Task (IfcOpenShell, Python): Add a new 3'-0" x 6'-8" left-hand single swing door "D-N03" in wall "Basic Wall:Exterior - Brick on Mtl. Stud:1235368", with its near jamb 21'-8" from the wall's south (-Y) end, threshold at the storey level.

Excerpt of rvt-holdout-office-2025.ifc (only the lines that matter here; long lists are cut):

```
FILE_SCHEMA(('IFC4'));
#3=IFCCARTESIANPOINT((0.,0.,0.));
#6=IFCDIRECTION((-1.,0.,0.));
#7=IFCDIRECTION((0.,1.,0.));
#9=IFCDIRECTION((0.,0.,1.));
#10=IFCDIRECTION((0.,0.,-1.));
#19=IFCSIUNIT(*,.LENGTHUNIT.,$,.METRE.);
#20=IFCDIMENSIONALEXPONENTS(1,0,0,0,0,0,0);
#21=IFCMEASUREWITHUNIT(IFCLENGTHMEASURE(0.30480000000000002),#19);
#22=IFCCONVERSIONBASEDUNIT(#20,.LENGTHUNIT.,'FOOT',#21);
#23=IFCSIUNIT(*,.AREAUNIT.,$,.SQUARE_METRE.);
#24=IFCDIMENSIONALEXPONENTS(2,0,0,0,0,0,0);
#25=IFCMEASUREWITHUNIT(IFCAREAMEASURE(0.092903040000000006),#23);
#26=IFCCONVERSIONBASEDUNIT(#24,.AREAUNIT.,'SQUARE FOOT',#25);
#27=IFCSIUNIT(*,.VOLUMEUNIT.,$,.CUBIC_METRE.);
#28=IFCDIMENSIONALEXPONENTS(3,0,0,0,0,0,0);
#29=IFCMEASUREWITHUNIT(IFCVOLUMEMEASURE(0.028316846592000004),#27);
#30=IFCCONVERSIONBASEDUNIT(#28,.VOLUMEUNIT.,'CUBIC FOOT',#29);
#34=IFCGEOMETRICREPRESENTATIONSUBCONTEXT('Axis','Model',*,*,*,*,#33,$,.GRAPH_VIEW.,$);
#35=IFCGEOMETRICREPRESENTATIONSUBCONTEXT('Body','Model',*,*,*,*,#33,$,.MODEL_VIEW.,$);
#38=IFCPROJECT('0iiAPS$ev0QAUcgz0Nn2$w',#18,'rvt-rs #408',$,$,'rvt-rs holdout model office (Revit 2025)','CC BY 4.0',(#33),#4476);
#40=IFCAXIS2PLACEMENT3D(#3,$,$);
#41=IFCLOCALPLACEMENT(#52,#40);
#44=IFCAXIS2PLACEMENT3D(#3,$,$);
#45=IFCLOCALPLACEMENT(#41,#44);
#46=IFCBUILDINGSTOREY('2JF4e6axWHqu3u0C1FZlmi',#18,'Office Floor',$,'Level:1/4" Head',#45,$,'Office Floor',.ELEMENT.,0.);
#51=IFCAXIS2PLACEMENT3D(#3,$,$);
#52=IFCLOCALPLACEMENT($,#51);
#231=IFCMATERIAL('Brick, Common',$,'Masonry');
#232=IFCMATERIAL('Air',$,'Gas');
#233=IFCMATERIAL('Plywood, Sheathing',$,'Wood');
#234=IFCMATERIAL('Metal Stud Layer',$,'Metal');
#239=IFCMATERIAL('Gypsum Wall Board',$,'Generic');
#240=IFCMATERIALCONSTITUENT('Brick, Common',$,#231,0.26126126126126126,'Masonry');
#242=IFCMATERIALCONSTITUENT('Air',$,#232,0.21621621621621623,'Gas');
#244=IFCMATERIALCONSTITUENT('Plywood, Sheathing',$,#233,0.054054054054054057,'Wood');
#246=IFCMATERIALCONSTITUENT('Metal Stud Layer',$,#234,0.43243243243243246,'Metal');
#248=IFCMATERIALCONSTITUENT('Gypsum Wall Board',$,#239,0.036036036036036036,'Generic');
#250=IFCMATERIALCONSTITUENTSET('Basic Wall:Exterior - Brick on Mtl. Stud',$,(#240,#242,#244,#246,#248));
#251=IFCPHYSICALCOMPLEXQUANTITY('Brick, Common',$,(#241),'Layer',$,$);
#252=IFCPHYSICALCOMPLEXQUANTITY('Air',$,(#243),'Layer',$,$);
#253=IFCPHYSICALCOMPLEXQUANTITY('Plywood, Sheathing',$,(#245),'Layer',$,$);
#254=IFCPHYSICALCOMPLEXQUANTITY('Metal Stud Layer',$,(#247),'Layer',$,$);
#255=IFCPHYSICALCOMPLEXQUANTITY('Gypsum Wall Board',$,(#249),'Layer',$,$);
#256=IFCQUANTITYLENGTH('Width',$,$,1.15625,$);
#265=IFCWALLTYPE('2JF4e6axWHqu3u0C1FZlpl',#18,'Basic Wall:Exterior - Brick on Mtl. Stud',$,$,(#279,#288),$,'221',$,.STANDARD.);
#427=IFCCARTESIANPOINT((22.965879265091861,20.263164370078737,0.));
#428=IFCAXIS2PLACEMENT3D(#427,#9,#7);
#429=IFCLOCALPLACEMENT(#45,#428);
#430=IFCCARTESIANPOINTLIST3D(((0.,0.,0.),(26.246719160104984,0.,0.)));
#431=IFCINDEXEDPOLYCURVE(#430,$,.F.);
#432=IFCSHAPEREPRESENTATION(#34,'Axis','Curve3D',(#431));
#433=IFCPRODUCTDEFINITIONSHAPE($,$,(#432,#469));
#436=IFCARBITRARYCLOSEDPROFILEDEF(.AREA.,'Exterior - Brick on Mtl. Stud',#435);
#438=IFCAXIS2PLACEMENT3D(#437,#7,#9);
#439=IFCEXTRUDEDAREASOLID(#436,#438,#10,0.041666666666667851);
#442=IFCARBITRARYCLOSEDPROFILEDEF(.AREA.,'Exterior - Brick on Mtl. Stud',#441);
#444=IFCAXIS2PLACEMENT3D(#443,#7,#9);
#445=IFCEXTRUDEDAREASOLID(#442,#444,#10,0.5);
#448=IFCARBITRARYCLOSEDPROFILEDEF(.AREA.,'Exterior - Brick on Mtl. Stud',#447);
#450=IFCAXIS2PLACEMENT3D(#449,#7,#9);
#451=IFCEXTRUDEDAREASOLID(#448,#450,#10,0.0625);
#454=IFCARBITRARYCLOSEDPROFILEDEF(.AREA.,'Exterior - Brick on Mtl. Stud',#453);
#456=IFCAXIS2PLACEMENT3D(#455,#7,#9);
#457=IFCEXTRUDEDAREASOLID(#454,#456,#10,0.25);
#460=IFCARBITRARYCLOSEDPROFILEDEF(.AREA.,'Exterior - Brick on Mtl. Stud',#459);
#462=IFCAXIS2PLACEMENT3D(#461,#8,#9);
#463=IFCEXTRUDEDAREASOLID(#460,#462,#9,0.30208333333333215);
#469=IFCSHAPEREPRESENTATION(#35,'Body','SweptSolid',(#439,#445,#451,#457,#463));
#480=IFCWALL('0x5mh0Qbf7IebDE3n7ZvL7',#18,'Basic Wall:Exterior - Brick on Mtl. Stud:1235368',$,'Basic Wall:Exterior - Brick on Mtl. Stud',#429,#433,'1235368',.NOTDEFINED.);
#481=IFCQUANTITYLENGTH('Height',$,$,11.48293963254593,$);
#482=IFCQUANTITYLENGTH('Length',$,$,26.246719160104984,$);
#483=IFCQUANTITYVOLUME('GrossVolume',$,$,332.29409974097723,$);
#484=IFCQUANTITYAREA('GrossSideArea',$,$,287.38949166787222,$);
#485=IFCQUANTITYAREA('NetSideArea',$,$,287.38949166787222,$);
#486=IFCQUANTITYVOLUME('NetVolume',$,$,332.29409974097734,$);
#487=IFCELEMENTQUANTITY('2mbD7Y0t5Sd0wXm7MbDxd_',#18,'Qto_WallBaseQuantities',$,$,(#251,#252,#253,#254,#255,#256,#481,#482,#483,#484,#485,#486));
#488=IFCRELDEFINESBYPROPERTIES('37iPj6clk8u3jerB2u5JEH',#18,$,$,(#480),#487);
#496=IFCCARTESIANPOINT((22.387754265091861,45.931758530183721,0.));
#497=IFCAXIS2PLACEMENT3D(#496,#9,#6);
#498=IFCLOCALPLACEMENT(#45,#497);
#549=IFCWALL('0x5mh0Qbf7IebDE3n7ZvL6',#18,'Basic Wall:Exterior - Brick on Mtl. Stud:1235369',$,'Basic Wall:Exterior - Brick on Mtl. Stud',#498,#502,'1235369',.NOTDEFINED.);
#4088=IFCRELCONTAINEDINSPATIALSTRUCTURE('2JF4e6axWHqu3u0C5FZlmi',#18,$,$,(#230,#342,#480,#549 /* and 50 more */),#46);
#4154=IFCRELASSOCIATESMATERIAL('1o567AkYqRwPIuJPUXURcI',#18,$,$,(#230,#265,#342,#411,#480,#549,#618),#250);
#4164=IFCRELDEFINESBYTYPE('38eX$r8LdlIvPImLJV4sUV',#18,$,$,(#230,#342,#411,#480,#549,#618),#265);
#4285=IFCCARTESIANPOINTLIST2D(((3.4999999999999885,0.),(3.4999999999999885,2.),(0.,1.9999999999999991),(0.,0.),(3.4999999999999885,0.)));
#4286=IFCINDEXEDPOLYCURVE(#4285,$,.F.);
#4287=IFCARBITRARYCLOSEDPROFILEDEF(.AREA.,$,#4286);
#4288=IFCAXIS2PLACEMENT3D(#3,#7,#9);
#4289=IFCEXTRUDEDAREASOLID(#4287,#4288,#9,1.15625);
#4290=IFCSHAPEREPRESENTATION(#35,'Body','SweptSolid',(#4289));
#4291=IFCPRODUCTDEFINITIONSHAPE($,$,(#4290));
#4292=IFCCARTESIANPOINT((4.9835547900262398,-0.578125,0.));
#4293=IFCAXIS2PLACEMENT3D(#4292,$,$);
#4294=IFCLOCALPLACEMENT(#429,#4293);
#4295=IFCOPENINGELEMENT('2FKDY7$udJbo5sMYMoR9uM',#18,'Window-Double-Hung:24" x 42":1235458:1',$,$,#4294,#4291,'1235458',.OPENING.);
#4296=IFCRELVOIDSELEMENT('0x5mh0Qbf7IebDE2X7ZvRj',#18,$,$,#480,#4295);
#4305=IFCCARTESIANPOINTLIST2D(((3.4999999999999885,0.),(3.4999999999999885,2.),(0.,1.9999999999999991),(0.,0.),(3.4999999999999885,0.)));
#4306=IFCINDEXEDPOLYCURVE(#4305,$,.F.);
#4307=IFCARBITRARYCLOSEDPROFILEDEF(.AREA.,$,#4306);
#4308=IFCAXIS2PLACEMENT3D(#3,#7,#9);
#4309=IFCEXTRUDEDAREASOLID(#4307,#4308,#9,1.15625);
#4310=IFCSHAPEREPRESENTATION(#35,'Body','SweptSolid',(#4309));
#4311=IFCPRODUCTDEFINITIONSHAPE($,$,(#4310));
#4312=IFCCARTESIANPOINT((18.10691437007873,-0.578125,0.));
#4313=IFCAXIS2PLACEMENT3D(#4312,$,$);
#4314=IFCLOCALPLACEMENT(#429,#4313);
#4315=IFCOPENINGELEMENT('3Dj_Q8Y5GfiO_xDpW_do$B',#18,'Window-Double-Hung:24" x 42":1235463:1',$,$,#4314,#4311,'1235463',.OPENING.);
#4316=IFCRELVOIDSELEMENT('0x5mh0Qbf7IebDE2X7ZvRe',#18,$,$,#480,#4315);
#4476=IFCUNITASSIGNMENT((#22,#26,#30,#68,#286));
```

```python
import numpy as np
import ifcopenshell
import ifcopenshell.api.feature
import ifcopenshell.api.geometry
import ifcopenshell.api.pset
import ifcopenshell.api.root
import ifcopenshell.api.spatial
import ifcopenshell.geom
import ifcopenshell.util.element
import ifcopenshell.util.placement
import ifcopenshell.util.representation
import ifcopenshell.util.shape
import ifcopenshell.util.unit

model = ifcopenshell.open("rvt-holdout-office-2025.ifc")
unit_scale = ifcopenshell.util.unit.calculate_unit_scale(model)
area_scale = ifcopenshell.util.unit.calculate_unit_scale(model, "AREAUNIT")
volume_scale = ifcopenshell.util.unit.calculate_unit_scale(model, "VOLUMEUNIT")
settings = ifcopenshell.geom.settings()


def volume(element):
    """Net volume in cubic metres, openings subtracted."""
    shape = ifcopenshell.geom.create_shape(settings, element)
    return ifcopenshell.util.shape.get_volume(shape.geometry)


wall = model.by_id(480)
storey = ifcopenshell.util.element.get_container(wall, ifc_class="IfcBuildingStorey")
context = ifcopenshell.util.representation.get_context(model, "Model", "Body", "MODEL_VIEW")
before = volume(wall)

width, height, from_end, sill = 0.9144, 2.032, 6.604, 0.0  # metres

# The wall runs along its own X axis, and the end named is its -X end.
wall_shape = ifcopenshell.geom.create_shape(settings, wall)
x, y, z = ifcopenshell.util.shape.get_vertices(wall_shape.geometry).T
start = x.min() + from_end
face, thickness = float(y.min()), float(y.max() - y.min())
wall_matrix = ifcopenshell.util.placement.get_local_placement(wall.ObjectPlacement)
level = ifcopenshell.util.placement.get_local_placement(storey.ObjectPlacement)[2, 3]


def in_wall(x, y):
    """Placement at x, y metres in the wall's axes, at sill height."""
    matrix = wall_matrix.copy()
    matrix[:, 3] = wall_matrix @ np.array([x / unit_scale, y / unit_scale, 0.0, 1.0])
    matrix[2, 3] = level + sill / unit_scale
    return matrix


# Opening: a box that overshoots both wall faces by 50 mm.
opening = ifcopenshell.api.root.create_entity(model, ifc_class="IfcOpeningElement", predefined_type="OPENING")
box = ifcopenshell.api.geometry.add_wall_representation(
    model, context=context, length=width, height=height, thickness=thickness + 0.1
)
ifcopenshell.api.geometry.assign_representation(model, product=opening, representation=box)
ifcopenshell.api.geometry.edit_object_placement(model, product=opening, matrix=in_wall(start, face - 0.05), is_si=False)
ifcopenshell.api.feature.add_feature(model, feature=opening, element=wall)

door = ifcopenshell.api.root.create_entity(model, ifc_class="IfcDoor", name="D-N03", predefined_type="DOOR")
door.OverallWidth, door.OverallHeight = width / unit_scale, height / unit_scale
door.OperationType = "SINGLE_SWING_LEFT"
body = ifcopenshell.api.geometry.add_door_representation(
    model,
    context=context,
    overall_width=door.OverallWidth,
    overall_height=door.OverallHeight,
    operation_type="SINGLE_SWING_LEFT",
    lining_properties={"LiningDepth": thickness / unit_scale, "ThresholdDepth": thickness / unit_scale},
)
ifcopenshell.api.geometry.assign_representation(model, product=door, representation=body)
ifcopenshell.api.spatial.assign_container(model, products=[door], relating_structure=storey)
ifcopenshell.api.feature.add_filling(model, opening=opening, element=door)

# The lining spans the wall, so the door starts at the wall face.
ifcopenshell.api.geometry.edit_object_placement(model, product=door, matrix=in_wall(start, face), is_si=False)

after = volume(wall)

# Update the wall's stored quantities.
qto = model.by_id(ifcopenshell.util.element.get_pset(wall, "Qto_WallBaseQuantities", should_inherit=False)["id"])
ifcopenshell.api.pset.edit_qto(model, qto=qto, properties={
    "NetSideArea": after / thickness / area_scale,
    "NetVolume": after / volume_scale,
})

print(f"wall volume {before:.3f} -> {after:.3f} m3")

model.write("rvt-holdout-office-2025_edited.ifc")
```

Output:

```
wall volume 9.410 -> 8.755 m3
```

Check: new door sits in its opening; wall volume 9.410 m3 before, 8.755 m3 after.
